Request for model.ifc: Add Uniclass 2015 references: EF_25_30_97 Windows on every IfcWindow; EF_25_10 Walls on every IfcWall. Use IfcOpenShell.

First a look at what the model holds.

```python
import ifcopenshell

model = ifcopenshell.open("model.ifc")
print(model.schema)
print("classifications:", [c.Name for c in model.by_type("IfcClassification")])
for ifc_class in ("IfcDoor", "IfcRoof", "IfcStair", "IfcWall", "IfcWindow"):
    print(ifc_class, len(model.by_type(ifc_class)))
```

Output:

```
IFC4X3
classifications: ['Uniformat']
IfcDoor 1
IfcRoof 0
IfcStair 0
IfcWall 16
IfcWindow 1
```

```python
import ifcopenshell
import ifcopenshell.api.classification

model = ifcopenshell.open("model.ifc")

system = ifcopenshell.api.classification.add_classification(model, classification="Uniclass 2015")

codes = {
    "IfcWindow": ("EF_25_30_97", "Windows"),
    "IfcWall": ("EF_25_10", "Walls"),
}
for ifc_class, (code, name) in codes.items():
    products = model.by_type(ifc_class)
    ifcopenshell.api.classification.add_reference(
        model, products=products, classification=system, identification=code, name=name
    )
    print(code, len(products))

model.write("model_updated.ifc")
```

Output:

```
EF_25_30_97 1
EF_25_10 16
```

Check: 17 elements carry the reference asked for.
